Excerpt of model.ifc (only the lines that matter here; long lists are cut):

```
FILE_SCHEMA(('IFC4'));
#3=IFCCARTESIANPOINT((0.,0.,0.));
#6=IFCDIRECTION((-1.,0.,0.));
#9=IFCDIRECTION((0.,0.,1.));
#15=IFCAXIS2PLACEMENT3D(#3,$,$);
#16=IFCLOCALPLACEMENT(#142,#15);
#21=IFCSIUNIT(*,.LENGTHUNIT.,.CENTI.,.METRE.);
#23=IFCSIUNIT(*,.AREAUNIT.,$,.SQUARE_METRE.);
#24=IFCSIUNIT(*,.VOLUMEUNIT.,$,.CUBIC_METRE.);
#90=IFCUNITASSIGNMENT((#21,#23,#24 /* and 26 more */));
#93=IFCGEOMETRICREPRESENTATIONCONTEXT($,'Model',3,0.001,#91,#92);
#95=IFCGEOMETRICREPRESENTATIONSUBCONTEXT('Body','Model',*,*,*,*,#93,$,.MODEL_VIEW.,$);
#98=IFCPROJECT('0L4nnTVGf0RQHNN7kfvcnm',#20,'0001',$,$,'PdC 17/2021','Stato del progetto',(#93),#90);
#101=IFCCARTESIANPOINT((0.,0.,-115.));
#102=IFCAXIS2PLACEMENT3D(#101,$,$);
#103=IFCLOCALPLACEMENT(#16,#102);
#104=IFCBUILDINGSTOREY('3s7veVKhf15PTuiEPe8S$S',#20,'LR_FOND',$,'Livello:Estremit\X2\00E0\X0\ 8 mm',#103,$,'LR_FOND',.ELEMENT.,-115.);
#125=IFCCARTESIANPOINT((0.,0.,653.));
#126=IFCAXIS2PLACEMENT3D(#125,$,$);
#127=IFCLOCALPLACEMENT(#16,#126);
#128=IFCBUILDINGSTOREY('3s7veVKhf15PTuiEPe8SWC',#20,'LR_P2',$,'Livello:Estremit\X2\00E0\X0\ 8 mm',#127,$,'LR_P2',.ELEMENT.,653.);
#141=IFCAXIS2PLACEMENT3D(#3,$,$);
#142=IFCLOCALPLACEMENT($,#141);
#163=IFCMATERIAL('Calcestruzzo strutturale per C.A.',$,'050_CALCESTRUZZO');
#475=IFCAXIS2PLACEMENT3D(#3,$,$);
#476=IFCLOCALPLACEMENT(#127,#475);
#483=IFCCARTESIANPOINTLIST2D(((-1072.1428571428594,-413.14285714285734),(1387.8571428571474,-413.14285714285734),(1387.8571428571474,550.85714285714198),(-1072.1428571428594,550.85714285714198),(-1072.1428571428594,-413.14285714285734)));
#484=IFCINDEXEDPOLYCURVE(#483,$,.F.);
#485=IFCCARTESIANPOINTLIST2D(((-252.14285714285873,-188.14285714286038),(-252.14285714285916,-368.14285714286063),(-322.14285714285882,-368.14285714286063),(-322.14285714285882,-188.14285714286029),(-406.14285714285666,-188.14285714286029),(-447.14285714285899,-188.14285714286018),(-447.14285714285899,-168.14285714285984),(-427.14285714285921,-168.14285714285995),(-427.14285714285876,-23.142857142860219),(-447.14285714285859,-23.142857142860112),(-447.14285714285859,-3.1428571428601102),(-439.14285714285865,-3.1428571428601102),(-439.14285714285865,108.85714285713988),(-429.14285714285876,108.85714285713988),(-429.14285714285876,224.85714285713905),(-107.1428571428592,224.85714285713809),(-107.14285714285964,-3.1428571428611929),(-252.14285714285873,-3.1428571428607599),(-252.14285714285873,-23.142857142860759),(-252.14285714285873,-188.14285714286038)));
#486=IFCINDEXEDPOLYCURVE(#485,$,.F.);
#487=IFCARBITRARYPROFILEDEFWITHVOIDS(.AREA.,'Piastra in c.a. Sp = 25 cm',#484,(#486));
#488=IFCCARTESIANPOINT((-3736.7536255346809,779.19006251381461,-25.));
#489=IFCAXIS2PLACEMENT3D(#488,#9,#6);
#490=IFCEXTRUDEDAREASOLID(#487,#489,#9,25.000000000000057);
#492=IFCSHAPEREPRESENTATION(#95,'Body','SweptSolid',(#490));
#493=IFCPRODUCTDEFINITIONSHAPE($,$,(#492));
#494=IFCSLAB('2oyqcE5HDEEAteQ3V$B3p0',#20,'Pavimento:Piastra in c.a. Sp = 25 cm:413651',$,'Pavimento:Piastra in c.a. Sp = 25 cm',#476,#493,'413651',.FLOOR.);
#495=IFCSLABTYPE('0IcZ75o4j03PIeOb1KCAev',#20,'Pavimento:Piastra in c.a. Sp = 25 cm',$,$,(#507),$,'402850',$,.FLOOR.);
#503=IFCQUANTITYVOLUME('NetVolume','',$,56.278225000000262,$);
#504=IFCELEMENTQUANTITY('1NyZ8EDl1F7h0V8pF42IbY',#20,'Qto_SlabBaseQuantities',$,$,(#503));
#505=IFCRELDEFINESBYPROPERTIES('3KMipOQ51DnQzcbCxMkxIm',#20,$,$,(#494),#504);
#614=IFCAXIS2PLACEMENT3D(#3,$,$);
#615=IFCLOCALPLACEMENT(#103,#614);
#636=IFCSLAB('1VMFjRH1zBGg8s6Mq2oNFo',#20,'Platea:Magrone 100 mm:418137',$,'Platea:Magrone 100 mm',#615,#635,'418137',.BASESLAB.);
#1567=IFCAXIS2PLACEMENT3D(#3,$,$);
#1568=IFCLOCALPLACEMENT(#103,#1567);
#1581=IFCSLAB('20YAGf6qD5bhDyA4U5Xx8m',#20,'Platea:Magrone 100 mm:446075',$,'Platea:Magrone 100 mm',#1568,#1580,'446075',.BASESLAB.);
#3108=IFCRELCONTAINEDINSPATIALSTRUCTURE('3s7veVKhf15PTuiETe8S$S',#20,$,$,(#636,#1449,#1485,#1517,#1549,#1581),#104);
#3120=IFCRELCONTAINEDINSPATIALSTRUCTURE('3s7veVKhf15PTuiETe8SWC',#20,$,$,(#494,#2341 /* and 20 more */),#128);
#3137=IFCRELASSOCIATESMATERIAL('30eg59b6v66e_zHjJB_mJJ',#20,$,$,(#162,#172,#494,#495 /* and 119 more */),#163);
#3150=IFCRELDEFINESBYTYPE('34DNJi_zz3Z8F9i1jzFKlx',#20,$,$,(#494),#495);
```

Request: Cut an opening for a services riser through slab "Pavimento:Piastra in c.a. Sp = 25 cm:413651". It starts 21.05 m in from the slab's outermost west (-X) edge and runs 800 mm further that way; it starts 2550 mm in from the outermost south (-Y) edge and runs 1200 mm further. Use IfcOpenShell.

```python
import numpy as np
import ifcopenshell
import ifcopenshell.api.feature
import ifcopenshell.api.geometry
import ifcopenshell.api.pset
import ifcopenshell.api.root
import ifcopenshell.geom
import ifcopenshell.util.element
import ifcopenshell.util.placement
import ifcopenshell.util.representation
import ifcopenshell.util.shape
import ifcopenshell.util.unit

model = ifcopenshell.open("model.ifc")
unit_scale = ifcopenshell.util.unit.calculate_unit_scale(model)
volume_scale = ifcopenshell.util.unit.calculate_unit_scale(model, "VOLUMEUNIT")
settings = ifcopenshell.geom.settings()


def volume(element):
    """Net volume in cubic metres, openings subtracted."""
    shape = ifcopenshell.geom.create_shape(settings, element)
    return ifcopenshell.util.shape.get_volume(shape.geometry)


slab = model.by_id(494)
before = volume(slab)

# Extent in the slab's own axes, in metres. The edges named are its -X and -Y sides.
slab_shape = ifcopenshell.geom.create_shape(settings, slab)
vertices = ifcopenshell.util.shape.get_vertices(slab_shape.geometry)
x_min, y_min, bottom = vertices.min(axis=0)
top = vertices[:, 2].max()

opening = ifcopenshell.api.root.create_entity(model, ifc_class="IfcOpeningElement", name="Services riser opening", predefined_type="OPENING")
context = ifcopenshell.util.representation.get_context(model, "Model", "Body", "MODEL_VIEW")
width, depth = 0.8, 1.2
outline = [(0.0, 0.0), (width, 0.0), (width, depth), (0.0, depth), (0.0, 0.0)]
# Overshoot both faces by 50 mm so the cut is clean.
shape = ifcopenshell.api.geometry.add_slab_representation(
    model, context=context, depth=top - bottom + 0.1, polyline=outline
)
ifcopenshell.api.geometry.assign_representation(model, product=opening, representation=shape)

matrix = ifcopenshell.util.placement.get_local_placement(slab.ObjectPlacement)
matrix[:, 3] = matrix @ np.append(np.array([x_min + 21.05, y_min + 2.55, bottom - 0.05]) / unit_scale, 1.0)
ifcopenshell.api.geometry.edit_object_placement(model, product=opening, matrix=matrix, is_si=False)
ifcopenshell.api.feature.add_feature(model, feature=opening, element=slab)

after = volume(slab)

# Update the slab's stored quantities.
qto = model.by_id(ifcopenshell.util.element.get_pset(slab, "Qto_SlabBaseQuantities", should_inherit=False)["id"])
ifcopenshell.api.pset.edit_qto(model, qto=qto, properties={"NetVolume": after / volume_scale})

print(f"slab volume {before:.3f} -> {after:.3f} m3")

model.write("model_updated.ifc")
```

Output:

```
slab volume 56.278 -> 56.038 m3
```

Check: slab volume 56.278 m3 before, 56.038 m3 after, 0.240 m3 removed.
